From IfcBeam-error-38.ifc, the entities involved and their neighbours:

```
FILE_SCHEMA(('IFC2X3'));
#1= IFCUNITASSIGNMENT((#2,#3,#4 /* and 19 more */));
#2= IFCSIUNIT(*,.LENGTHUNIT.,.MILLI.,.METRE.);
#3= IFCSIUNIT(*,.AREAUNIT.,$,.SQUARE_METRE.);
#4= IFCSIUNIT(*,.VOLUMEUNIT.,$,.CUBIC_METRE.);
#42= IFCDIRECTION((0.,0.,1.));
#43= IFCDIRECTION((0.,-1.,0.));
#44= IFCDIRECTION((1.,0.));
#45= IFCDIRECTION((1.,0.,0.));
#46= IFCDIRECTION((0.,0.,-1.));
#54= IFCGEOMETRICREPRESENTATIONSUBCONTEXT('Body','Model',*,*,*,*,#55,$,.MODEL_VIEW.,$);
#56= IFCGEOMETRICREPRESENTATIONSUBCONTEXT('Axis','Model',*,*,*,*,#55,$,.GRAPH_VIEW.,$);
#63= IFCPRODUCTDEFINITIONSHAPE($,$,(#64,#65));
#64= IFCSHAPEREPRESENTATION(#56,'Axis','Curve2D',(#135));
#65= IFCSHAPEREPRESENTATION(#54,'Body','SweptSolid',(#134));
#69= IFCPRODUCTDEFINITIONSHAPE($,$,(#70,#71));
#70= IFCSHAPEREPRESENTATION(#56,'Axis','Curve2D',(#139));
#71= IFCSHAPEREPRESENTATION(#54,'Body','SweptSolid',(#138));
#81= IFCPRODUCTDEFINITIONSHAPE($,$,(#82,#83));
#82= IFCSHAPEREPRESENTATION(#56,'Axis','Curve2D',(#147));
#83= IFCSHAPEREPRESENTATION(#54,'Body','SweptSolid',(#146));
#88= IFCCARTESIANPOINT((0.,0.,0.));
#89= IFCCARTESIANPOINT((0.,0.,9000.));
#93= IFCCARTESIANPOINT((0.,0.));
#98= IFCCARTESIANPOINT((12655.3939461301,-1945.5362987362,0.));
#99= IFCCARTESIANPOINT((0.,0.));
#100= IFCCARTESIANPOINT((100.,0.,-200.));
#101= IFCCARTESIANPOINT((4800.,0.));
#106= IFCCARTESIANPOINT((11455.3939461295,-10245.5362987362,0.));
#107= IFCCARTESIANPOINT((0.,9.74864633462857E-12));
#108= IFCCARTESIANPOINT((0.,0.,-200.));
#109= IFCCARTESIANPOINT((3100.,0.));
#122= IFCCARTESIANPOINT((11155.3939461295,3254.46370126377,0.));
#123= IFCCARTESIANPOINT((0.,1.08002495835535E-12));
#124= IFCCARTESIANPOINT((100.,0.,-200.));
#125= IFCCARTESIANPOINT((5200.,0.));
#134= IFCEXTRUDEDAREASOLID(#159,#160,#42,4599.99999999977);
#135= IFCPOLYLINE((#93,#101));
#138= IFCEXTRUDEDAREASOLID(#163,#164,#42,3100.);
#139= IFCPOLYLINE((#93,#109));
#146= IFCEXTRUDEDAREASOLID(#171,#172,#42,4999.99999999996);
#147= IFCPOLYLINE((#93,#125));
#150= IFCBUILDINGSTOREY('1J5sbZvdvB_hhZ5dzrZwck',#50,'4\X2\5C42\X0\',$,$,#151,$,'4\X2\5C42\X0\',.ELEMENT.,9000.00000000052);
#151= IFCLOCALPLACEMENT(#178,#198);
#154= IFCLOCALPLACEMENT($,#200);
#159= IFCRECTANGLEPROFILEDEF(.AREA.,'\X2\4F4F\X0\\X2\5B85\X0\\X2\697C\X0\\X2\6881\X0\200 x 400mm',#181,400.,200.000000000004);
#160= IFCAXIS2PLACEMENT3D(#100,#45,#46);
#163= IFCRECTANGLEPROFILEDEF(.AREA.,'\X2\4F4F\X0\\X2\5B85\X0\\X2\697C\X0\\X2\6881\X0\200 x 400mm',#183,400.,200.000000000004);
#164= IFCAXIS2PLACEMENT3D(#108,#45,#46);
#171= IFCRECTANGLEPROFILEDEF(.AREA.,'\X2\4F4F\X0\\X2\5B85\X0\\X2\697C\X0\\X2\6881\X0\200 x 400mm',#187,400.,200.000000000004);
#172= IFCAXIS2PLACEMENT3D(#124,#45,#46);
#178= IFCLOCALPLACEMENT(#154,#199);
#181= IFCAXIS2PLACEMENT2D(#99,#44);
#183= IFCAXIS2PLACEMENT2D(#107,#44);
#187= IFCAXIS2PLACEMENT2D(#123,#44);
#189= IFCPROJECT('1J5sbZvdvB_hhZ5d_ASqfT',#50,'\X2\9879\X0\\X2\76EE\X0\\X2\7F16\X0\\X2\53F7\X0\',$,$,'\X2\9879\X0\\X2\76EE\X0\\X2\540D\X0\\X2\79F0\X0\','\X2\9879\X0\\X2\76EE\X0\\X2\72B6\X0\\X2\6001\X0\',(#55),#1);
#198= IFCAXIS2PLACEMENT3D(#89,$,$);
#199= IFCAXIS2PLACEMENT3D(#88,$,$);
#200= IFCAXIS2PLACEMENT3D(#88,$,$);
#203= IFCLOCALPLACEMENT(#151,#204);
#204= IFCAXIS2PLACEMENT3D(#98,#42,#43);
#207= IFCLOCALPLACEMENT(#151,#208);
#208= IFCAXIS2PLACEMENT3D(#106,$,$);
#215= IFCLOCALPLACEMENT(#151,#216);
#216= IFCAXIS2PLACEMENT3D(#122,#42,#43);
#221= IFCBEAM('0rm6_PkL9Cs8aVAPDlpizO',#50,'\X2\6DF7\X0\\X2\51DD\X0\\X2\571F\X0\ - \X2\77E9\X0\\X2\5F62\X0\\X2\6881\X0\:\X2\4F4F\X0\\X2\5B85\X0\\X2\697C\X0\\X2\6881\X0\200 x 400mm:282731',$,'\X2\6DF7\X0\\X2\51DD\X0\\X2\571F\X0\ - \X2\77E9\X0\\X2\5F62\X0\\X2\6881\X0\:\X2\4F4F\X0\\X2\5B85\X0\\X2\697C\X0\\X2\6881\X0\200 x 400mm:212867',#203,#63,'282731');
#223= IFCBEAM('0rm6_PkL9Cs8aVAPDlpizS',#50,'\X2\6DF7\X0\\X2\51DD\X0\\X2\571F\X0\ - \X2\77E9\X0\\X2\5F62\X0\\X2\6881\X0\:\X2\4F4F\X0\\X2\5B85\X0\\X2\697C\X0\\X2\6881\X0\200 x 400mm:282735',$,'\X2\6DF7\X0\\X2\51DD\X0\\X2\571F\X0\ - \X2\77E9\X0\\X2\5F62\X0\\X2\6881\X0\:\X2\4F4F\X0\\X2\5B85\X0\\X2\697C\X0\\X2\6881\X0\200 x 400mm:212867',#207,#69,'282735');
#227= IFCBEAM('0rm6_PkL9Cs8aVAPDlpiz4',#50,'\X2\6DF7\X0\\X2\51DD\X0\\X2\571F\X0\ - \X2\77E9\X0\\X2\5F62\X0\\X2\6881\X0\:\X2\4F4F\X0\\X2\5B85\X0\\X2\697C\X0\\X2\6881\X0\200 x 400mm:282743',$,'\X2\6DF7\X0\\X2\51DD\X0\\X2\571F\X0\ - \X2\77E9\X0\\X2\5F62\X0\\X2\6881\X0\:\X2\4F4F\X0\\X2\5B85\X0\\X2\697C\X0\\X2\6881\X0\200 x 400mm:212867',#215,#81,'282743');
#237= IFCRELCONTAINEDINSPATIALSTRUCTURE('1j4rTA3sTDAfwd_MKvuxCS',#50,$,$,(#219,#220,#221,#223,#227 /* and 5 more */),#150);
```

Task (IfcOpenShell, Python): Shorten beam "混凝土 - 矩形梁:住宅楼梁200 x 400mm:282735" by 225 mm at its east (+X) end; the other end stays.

```python
import numpy as np
import ifcopenshell
import ifcopenshell.util.representation

model = ifcopenshell.open("IfcBeam-error-38.ifc")

member = model.by_guid("0rm6_PkL9Cs8aVAPDlpizS")
change = -225.0

# The extrusion runs towards the end named, so only its depth changes.
body = ifcopenshell.util.representation.get_representation(member, "Model", "Body")
solid = body.Items[0]
old_length = solid.Depth
solid.Depth += change

# Move the axis end point with it.
axis = next(r for r in member.Representation.Representations if r.RepresentationIdentifier == "Axis").Items[0]
start, end = (np.array(p.Coordinates) for p in axis.Points)
end = end + (end - start) / np.linalg.norm(end - start) * change
point = model.createIfcCartesianPoint(end.tolist())
axis.Points = [axis.Points[0], point]

print(f"length {old_length:g} -> {solid.Depth:g}")

model.write("IfcBeam-error-38_updated.ifc")
```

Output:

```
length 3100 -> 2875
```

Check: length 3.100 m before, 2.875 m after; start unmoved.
